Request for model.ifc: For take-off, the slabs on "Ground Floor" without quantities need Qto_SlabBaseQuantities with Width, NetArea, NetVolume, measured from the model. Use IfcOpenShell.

First a look at what the model holds.

```python
import ifcopenshell
import ifcopenshell.util.element
import ifcopenshell.util.unit

model = ifcopenshell.open("model.ifc")
print(model.schema)
for unit_type in ("LENGTHUNIT", "AREAUNIT", "VOLUMEUNIT"):
    print(unit_type, ifcopenshell.util.unit.calculate_unit_scale(model, unit_type))
storey = next(s for s in model.by_type("IfcBuildingStorey") if s.Name == "Ground Floor")
slabs = [e for e in ifcopenshell.util.element.get_decomposition(storey) if e.is_a("IfcSlab")]
for e in sorted(slabs, key=lambda e: e.id()):
    print(e.id(), e.is_a(), e.Name, list(ifcopenshell.util.element.get_psets(e, qtos_only=True)), sep=" | ")
```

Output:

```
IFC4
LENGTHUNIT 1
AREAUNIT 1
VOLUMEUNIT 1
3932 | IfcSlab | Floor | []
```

```python
import ifcopenshell
import ifcopenshell.api.pset
import ifcopenshell.geom
import ifcopenshell.util.element
import ifcopenshell.util.shape
import ifcopenshell.util.unit

model = ifcopenshell.open("model.ifc")
unit_scale = ifcopenshell.util.unit.calculate_unit_scale(model)
area_scale = ifcopenshell.util.unit.calculate_unit_scale(model, "AREAUNIT")
volume_scale = ifcopenshell.util.unit.calculate_unit_scale(model, "VOLUMEUNIT")
settings = ifcopenshell.geom.settings()

storey = next(s for s in model.by_type("IfcBuildingStorey") if s.Name == "Ground Floor")
slabs = [e for e in ifcopenshell.util.element.get_decomposition(storey) if e.is_a("IfcSlab")]

for e in sorted(slabs, key=lambda e: e.id()):
    if ifcopenshell.util.element.get_psets(e, qtos_only=True, should_inherit=False):
        continue
    # Geometry comes back in metres, in the element's own axes.
    shape = ifcopenshell.geom.create_shape(settings, e)
    values = {
        "Width": ifcopenshell.util.shape.get_z(shape.geometry) / unit_scale,
        "NetArea": ifcopenshell.util.shape.get_footprint_area(shape.geometry) / area_scale,
        "NetVolume": ifcopenshell.util.shape.get_volume(shape.geometry) / volume_scale,
    }
    qto = ifcopenshell.api.pset.add_qto(model, product=e, name="Qto_SlabBaseQuantities")
    ifcopenshell.api.pset.edit_qto(model, qto=qto, properties=values)
    print(e.id(), {k: round(v, 3) for k, v in values.items()})

model.write("model-out.ifc")
```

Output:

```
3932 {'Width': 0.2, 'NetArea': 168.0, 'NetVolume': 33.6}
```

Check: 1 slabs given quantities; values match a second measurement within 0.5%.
